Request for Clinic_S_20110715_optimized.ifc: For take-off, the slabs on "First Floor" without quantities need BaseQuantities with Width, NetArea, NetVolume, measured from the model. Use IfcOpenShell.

First a look at what the model holds.

```python
import ifcopenshell
import ifcopenshell.util.element
import ifcopenshell.util.unit

model = ifcopenshell.open("Clinic_S_20110715_optimized.ifc")
print(model.schema)
for unit_type in ("LENGTHUNIT", "AREAUNIT", "VOLUMEUNIT"):
    print(unit_type, ifcopenshell.util.unit.calculate_unit_scale(model, unit_type))
storey = next(s for s in model.by_type("IfcBuildingStorey") if s.Name == "First Floor")
slabs = [e for e in ifcopenshell.util.element.get_decomposition(storey) if e.is_a("IfcSlab")]
for e in sorted(slabs, key=lambda e: e.id()):
    print(e.id(), e.is_a(), e.Name, list(ifcopenshell.util.element.get_psets(e, qtos_only=True)), sep=" | ")
```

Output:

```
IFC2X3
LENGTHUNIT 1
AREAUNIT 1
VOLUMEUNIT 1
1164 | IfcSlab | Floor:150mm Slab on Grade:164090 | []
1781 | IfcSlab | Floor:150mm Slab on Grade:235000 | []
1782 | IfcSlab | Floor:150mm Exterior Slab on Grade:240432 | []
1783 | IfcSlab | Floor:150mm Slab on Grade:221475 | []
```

```python
import ifcopenshell
import ifcopenshell.api.pset
import ifcopenshell.geom
import ifcopenshell.util.element
import ifcopenshell.util.shape
import ifcopenshell.util.unit

model = ifcopenshell.open("Clinic_S_20110715_optimized.ifc")
unit_scale = ifcopenshell.util.unit.calculate_unit_scale(model)
area_scale = ifcopenshell.util.unit.calculate_unit_scale(model, "AREAUNIT")
volume_scale = ifcopenshell.util.unit.calculate_unit_scale(model, "VOLUMEUNIT")
settings = ifcopenshell.geom.settings()

storey = next(s for s in model.by_type("IfcBuildingStorey") if s.Name == "First Floor")
slabs = [e for e in ifcopenshell.util.element.get_decomposition(storey) if e.is_a("IfcSlab")]

for e in sorted(slabs, key=lambda e: e.id()):
    if ifcopenshell.util.element.get_psets(e, qtos_only=True, should_inherit=False):
        continue
    # Geometry comes back in metres, in the element's own axes.
    shape = ifcopenshell.geom.create_shape(settings, e)
    values = {
        "Width": ifcopenshell.util.shape.get_z(shape.geometry) / unit_scale,
        "NetArea": ifcopenshell.util.shape.get_footprint_area(shape.geometry) / area_scale,
        "NetVolume": ifcopenshell.util.shape.get_volume(shape.geometry) / volume_scale,
    }
    qto = ifcopenshell.api.pset.add_qto(model, product=e, name="BaseQuantities")
    ifcopenshell.api.pset.edit_qto(model, qto=qto, properties=values)
    print(e.id(), {k: round(v, 3) for k, v in values.items()})

model.write("Clinic_S_20110715_optimized_v2.ifc")
```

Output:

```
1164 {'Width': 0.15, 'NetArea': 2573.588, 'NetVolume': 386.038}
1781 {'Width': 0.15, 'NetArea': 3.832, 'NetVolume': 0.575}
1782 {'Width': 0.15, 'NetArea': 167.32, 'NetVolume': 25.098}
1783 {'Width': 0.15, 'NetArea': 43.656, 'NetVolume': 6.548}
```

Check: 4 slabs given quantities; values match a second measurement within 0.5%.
